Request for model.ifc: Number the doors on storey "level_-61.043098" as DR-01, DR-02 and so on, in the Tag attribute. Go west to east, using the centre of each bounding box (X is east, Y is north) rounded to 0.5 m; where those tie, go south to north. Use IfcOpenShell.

First a look at what the model holds.

```python
import ifcopenshell
import ifcopenshell.util.element
import ifcopenshell.util.placement

model = ifcopenshell.open("model.ifc")
print(model.schema)
storey = next(s for s in model.by_type("IfcBuildingStorey") if s.Name == "level_-61.043098")
doors = [e for e in ifcopenshell.util.element.get_decomposition(storey) if e.is_a("IfcDoor")]
for e in sorted(doors, key=lambda e: e.id()):
    origin = ifcopenshell.util.placement.get_local_placement(e.ObjectPlacement)[:3, 3]
    print(e.id(), e.Tag, e.Name, origin.round(2) + 0.0, sep=" | ")
```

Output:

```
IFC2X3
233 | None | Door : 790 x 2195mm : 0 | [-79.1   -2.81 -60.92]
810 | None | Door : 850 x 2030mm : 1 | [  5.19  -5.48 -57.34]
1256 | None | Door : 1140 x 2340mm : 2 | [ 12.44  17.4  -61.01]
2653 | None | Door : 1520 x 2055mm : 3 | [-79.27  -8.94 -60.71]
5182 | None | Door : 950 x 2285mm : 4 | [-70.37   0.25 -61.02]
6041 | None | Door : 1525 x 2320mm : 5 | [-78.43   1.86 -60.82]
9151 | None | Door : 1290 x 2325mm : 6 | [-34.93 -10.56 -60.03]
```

```python
import ifcopenshell
import ifcopenshell.geom
import ifcopenshell.util.element
import ifcopenshell.util.shape

model = ifcopenshell.open("model.ifc")
settings = ifcopenshell.geom.settings()
settings.set("use-world-coords", True)


def centre(element):
    shape = ifcopenshell.geom.create_shape(settings, element)
    return ifcopenshell.util.shape.get_bbox_centroid(shape.geometry)


storey = next(s for s in model.by_type("IfcBuildingStorey") if s.Name == "level_-61.043098")
doors = [e for e in ifcopenshell.util.element.get_decomposition(storey) if e.is_a("IfcDoor")]

# Insertion points can sit at a corner or the storey origin, so sort by the geometry (in metres).
centres = {e: centre(e) for e in doors}
doors.sort(key=lambda e: (round(centres[e][0] / 0.5), centres[e][1]))

for i, e in enumerate(doors, start=1):
    number = f"DR-{i:02d}"
    e.Tag = number
    print(e.id(), number)

model.write("model_edited.ifc")
```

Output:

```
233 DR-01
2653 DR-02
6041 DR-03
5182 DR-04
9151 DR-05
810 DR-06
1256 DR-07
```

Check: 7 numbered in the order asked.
